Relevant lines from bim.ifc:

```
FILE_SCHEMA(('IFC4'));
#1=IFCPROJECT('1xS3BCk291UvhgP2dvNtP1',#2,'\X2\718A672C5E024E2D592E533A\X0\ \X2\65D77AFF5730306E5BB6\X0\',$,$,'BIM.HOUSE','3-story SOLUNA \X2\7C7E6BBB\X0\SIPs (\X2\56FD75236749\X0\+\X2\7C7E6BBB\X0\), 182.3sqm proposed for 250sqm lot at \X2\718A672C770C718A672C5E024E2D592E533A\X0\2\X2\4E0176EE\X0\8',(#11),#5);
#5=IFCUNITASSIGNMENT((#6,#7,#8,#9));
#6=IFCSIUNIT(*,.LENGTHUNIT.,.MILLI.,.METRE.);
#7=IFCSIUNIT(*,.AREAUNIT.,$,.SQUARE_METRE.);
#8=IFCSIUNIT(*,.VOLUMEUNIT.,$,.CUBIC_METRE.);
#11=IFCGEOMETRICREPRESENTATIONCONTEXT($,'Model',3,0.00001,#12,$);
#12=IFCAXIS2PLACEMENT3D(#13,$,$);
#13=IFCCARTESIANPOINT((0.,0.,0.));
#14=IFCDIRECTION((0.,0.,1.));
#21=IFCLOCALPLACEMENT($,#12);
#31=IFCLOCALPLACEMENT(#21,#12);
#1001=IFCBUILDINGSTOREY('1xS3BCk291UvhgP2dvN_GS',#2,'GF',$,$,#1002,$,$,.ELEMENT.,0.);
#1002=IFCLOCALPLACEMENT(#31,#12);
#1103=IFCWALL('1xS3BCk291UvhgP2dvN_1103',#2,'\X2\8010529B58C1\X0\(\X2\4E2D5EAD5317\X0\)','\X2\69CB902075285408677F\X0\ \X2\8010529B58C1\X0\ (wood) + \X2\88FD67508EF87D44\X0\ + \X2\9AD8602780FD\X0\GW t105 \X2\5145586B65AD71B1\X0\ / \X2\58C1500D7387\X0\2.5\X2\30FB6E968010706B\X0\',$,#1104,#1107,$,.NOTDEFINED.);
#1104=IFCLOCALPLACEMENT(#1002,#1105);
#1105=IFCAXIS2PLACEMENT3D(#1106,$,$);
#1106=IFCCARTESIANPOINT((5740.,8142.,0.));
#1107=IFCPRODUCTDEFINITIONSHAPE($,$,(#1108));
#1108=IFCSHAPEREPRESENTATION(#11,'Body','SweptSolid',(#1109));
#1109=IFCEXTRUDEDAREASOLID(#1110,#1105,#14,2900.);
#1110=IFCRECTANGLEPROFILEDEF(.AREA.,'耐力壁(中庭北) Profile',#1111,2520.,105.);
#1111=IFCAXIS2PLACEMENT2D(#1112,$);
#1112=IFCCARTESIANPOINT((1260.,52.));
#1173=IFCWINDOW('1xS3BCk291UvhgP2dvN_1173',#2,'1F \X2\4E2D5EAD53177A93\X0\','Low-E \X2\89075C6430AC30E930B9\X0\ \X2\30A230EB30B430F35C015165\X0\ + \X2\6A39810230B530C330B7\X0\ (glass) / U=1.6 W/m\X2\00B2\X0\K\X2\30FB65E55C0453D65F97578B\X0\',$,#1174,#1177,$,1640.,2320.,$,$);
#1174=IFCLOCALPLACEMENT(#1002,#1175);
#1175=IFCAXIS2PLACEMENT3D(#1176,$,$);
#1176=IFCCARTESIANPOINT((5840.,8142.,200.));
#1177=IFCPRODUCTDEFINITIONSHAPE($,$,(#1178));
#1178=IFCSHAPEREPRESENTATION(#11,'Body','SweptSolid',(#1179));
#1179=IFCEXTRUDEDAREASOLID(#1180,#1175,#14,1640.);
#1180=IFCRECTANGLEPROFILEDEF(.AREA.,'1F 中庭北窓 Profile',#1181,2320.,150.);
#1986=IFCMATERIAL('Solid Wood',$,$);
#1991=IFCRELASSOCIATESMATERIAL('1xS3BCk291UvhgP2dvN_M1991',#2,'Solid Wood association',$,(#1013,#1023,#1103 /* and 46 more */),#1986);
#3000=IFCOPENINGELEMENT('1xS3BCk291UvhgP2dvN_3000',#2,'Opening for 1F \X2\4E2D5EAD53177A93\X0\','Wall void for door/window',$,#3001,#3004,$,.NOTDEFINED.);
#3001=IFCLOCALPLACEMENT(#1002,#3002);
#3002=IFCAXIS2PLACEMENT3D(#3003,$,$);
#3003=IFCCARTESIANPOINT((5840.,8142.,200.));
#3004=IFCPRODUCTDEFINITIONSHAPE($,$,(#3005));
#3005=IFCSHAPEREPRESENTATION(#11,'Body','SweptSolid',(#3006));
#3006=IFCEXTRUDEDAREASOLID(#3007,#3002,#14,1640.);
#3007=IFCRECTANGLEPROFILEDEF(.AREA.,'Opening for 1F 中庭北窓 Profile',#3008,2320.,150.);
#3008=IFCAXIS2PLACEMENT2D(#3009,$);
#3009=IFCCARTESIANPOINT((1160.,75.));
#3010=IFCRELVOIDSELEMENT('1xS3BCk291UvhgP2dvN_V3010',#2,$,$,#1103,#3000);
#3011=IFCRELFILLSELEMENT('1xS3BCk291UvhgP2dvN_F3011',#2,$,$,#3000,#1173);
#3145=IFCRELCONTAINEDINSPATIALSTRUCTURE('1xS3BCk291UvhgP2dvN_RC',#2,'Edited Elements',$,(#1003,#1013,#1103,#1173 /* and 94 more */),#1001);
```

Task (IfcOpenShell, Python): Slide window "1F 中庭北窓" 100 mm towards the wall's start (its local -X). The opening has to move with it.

```python
import ifcopenshell
import ifcopenshell.api.geometry
import ifcopenshell.util.placement
import ifcopenshell.util.unit

model = ifcopenshell.open("bim.ifc")
unit_scale = ifcopenshell.util.unit.calculate_unit_scale(model)

window = model.by_id(1173)
opening = window.FillsVoids[0].RelatingOpeningElement
wall = opening.VoidsElements[0].RelatingBuildingElement

wall_matrix = ifcopenshell.util.placement.get_local_placement(wall.ObjectPlacement)
shift = wall_matrix[:3, 0] * -0.1 / unit_scale
before = ifcopenshell.util.placement.get_local_placement(window.ObjectPlacement)[:3, 3].copy()

# The window is not placed relative to its opening, so move both.
for product in (opening, window):
    matrix = ifcopenshell.util.placement.get_local_placement(product.ObjectPlacement)
    matrix[:3, 3] += shift
    ifcopenshell.api.geometry.edit_object_placement(model, product=product, matrix=matrix, is_si=False)

after = ifcopenshell.util.placement.get_local_placement(window.ObjectPlacement)[:3, 3]
print("window moved by", (after - before).round(3) + 0.0)

model.write("bim_rev.ifc")
```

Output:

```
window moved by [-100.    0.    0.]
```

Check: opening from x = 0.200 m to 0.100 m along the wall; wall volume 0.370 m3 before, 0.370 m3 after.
